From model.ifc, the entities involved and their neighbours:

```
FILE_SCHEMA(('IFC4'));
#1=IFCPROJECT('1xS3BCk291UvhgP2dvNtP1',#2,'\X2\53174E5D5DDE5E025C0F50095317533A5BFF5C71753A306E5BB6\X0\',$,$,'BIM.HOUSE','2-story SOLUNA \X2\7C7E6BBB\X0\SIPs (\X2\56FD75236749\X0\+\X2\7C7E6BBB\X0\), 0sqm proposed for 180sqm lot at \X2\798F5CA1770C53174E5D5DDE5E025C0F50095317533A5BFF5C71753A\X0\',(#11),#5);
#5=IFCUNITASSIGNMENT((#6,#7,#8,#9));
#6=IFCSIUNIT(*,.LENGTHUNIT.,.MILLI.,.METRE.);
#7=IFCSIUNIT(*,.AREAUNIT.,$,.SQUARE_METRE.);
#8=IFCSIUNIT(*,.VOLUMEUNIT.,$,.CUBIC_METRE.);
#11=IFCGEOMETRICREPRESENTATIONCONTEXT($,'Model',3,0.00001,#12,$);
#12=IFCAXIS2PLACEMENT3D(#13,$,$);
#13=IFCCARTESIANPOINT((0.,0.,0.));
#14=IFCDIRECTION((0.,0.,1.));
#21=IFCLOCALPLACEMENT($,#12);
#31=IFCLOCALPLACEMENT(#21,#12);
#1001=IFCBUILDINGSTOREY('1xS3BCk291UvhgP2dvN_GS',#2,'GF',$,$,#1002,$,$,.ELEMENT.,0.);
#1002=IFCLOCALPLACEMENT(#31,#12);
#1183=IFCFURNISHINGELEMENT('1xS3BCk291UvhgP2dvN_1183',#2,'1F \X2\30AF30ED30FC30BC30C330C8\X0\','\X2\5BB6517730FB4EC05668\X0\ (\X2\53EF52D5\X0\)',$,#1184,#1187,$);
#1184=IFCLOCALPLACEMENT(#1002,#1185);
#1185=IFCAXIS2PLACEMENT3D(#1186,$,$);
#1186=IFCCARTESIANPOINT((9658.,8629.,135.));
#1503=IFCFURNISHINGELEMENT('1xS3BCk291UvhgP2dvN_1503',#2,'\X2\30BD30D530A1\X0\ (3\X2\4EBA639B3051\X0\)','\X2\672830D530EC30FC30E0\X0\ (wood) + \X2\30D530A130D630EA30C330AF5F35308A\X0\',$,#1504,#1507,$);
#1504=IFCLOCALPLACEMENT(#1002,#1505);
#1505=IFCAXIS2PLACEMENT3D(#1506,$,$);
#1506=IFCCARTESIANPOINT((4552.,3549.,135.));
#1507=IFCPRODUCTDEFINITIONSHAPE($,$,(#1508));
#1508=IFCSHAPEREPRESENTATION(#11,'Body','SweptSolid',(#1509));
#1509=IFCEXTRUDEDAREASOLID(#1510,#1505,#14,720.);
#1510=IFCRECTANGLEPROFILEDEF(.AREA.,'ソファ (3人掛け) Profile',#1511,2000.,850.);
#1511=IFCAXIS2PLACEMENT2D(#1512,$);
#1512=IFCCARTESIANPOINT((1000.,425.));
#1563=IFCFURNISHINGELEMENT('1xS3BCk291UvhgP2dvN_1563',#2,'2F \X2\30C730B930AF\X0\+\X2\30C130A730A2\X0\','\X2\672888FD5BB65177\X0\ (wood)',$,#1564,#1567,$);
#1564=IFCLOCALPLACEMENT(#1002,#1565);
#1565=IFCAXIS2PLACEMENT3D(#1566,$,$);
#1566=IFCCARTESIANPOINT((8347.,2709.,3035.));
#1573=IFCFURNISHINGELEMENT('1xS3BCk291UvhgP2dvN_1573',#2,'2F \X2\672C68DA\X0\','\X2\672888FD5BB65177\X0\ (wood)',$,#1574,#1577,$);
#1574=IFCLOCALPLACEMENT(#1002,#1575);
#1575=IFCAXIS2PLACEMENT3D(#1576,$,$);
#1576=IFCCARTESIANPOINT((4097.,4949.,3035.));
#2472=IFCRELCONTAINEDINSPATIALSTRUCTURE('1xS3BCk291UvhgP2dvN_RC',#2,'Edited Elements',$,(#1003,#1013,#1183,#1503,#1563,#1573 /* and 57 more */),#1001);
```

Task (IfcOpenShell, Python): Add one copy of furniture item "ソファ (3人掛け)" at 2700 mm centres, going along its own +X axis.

```python
import ifcopenshell
import ifcopenshell.api.geometry
import ifcopenshell.api.root
import ifcopenshell.util.element
import ifcopenshell.util.placement
import ifcopenshell.util.unit

model = ifcopenshell.open("model.ifc")
unit_scale = ifcopenshell.util.unit.calculate_unit_scale(model)


def reuse_history(source, copy):
    """copy_class also copies each property set's owner history, people and application; keep the originals."""
    for rel in copy.IsDefinedBy:
        if rel.is_a("IfcRelDefinesByProperties") and (history := rel.RelatingPropertyDefinition.OwnerHistory):
            rel.RelatingPropertyDefinition.OwnerHistory = source.OwnerHistory
            ifcopenshell.util.element.remove_deep2(model, history)


source = model.by_id(1503)
base = ifcopenshell.util.placement.get_local_placement(source.ObjectPlacement)
step = base[:3, 0] * 2.7 / unit_scale

for i in range(1, 2):
    copy = ifcopenshell.api.root.copy_class(model, product=source)
    copy.Representation = ifcopenshell.util.element.copy_deep(
        model, source.Representation, exclude=["IfcGeometricRepresentationContext", "IfcRepresentationMap"]
    )
    reuse_history(source, copy)
    matrix = base.copy()
    matrix[:3, 3] += i * step
    print("added at", matrix[:3, 3].round(3) + 0.0)
    ifcopenshell.api.geometry.edit_object_placement(model, product=copy, matrix=matrix, is_si=False)

model.write("model_v2.ifc")
```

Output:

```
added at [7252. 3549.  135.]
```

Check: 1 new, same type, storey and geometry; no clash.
